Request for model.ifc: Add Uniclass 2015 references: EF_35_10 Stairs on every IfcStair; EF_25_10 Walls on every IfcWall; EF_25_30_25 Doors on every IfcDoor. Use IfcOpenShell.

First a look at what the model holds.

```python
import ifcopenshell

model = ifcopenshell.open("model.ifc")
print(model.schema)
print("classifications:", [c.Name for c in model.by_type("IfcClassification")])
for ifc_class in ("IfcDoor", "IfcRoof", "IfcStair", "IfcWall", "IfcWindow"):
    print(ifc_class, len(model.by_type(ifc_class)))
```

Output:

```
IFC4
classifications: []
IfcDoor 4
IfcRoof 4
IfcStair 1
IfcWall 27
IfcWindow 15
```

```python
import ifcopenshell
import ifcopenshell.api.classification

model = ifcopenshell.open("model.ifc")

system = ifcopenshell.api.classification.add_classification(model, classification="Uniclass 2015")

codes = {
    "IfcStair": ("EF_35_10", "Stairs"),
    "IfcWall": ("EF_25_10", "Walls"),
    "IfcDoor": ("EF_25_30_25", "Doors"),
}
for ifc_class, (code, name) in codes.items():
    products = model.by_type(ifc_class)
    ifcopenshell.api.classification.add_reference(
        model, products=products, classification=system, identification=code, name=name
    )
    print(code, len(products))

model.write("model_v2.ifc")
```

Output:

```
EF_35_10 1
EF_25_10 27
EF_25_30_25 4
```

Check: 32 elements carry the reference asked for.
